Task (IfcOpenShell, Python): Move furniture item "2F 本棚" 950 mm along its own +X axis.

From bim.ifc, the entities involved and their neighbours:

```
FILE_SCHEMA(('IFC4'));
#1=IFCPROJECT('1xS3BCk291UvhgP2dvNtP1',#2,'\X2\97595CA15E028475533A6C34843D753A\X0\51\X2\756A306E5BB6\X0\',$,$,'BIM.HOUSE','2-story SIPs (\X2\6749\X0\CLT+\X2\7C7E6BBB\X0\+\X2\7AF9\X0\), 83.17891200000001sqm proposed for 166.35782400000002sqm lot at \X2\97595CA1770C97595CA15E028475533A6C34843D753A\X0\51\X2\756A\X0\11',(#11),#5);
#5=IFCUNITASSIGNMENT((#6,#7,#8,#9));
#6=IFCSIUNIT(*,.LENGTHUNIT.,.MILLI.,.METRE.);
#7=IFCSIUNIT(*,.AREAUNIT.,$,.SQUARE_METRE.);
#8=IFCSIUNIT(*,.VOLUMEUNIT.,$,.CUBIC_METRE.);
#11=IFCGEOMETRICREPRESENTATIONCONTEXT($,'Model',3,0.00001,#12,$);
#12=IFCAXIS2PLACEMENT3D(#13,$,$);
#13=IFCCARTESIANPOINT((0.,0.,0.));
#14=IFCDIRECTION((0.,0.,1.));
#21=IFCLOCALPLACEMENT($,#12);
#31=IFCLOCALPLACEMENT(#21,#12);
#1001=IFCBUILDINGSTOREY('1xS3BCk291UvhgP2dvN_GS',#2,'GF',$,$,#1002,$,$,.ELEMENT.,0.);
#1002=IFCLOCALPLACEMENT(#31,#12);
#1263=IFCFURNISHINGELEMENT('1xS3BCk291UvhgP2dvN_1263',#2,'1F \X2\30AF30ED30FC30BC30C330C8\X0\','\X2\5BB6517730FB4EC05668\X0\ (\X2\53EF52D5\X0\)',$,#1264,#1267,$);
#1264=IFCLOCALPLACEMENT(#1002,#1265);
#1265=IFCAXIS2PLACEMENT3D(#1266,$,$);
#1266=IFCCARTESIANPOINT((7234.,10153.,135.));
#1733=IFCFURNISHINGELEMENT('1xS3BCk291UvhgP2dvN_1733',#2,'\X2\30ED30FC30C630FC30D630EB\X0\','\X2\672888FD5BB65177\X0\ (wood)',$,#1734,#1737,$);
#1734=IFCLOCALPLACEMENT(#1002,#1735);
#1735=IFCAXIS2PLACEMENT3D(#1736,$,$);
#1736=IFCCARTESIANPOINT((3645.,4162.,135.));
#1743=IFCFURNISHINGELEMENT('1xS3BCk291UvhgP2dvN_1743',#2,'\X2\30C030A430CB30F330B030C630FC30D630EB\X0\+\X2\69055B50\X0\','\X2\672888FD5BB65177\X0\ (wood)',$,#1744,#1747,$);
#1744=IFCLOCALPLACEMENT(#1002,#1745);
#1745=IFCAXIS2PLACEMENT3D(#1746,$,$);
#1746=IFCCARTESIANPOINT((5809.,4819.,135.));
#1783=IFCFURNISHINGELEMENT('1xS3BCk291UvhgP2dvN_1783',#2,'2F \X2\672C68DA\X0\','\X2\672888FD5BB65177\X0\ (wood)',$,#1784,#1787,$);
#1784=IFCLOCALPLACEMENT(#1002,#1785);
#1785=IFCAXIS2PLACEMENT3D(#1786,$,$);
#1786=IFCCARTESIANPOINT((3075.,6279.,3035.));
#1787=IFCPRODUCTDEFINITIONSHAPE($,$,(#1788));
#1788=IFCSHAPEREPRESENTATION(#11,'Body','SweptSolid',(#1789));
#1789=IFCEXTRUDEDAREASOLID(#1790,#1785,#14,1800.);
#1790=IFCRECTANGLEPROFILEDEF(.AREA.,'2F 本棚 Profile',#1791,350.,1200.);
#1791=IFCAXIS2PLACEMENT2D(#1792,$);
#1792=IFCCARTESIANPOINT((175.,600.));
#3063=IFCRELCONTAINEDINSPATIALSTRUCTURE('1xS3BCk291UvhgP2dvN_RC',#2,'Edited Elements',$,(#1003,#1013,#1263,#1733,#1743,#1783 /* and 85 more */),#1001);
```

```python
import ifcopenshell
import ifcopenshell.api.geometry
import ifcopenshell.util.placement
import ifcopenshell.util.unit

model = ifcopenshell.open("bim.ifc")
unit_scale = ifcopenshell.util.unit.calculate_unit_scale(model)

item = model.by_guid("1xS3BCk291UvhgP2dvN_1783")
matrix = ifcopenshell.util.placement.get_local_placement(item.ObjectPlacement)
matrix[:3, 3] += matrix[:3, 0] * 0.95 / unit_scale
ifcopenshell.api.geometry.edit_object_placement(model, product=item, matrix=matrix, is_si=False)

print(ifcopenshell.util.placement.get_local_placement(item.ObjectPlacement).round(3) + 0.0)

model.write("bim_updated.ifc")
```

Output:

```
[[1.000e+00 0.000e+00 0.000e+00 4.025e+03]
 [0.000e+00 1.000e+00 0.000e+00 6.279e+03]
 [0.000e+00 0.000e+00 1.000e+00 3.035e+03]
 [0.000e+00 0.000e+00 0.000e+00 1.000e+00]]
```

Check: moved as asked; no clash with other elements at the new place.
